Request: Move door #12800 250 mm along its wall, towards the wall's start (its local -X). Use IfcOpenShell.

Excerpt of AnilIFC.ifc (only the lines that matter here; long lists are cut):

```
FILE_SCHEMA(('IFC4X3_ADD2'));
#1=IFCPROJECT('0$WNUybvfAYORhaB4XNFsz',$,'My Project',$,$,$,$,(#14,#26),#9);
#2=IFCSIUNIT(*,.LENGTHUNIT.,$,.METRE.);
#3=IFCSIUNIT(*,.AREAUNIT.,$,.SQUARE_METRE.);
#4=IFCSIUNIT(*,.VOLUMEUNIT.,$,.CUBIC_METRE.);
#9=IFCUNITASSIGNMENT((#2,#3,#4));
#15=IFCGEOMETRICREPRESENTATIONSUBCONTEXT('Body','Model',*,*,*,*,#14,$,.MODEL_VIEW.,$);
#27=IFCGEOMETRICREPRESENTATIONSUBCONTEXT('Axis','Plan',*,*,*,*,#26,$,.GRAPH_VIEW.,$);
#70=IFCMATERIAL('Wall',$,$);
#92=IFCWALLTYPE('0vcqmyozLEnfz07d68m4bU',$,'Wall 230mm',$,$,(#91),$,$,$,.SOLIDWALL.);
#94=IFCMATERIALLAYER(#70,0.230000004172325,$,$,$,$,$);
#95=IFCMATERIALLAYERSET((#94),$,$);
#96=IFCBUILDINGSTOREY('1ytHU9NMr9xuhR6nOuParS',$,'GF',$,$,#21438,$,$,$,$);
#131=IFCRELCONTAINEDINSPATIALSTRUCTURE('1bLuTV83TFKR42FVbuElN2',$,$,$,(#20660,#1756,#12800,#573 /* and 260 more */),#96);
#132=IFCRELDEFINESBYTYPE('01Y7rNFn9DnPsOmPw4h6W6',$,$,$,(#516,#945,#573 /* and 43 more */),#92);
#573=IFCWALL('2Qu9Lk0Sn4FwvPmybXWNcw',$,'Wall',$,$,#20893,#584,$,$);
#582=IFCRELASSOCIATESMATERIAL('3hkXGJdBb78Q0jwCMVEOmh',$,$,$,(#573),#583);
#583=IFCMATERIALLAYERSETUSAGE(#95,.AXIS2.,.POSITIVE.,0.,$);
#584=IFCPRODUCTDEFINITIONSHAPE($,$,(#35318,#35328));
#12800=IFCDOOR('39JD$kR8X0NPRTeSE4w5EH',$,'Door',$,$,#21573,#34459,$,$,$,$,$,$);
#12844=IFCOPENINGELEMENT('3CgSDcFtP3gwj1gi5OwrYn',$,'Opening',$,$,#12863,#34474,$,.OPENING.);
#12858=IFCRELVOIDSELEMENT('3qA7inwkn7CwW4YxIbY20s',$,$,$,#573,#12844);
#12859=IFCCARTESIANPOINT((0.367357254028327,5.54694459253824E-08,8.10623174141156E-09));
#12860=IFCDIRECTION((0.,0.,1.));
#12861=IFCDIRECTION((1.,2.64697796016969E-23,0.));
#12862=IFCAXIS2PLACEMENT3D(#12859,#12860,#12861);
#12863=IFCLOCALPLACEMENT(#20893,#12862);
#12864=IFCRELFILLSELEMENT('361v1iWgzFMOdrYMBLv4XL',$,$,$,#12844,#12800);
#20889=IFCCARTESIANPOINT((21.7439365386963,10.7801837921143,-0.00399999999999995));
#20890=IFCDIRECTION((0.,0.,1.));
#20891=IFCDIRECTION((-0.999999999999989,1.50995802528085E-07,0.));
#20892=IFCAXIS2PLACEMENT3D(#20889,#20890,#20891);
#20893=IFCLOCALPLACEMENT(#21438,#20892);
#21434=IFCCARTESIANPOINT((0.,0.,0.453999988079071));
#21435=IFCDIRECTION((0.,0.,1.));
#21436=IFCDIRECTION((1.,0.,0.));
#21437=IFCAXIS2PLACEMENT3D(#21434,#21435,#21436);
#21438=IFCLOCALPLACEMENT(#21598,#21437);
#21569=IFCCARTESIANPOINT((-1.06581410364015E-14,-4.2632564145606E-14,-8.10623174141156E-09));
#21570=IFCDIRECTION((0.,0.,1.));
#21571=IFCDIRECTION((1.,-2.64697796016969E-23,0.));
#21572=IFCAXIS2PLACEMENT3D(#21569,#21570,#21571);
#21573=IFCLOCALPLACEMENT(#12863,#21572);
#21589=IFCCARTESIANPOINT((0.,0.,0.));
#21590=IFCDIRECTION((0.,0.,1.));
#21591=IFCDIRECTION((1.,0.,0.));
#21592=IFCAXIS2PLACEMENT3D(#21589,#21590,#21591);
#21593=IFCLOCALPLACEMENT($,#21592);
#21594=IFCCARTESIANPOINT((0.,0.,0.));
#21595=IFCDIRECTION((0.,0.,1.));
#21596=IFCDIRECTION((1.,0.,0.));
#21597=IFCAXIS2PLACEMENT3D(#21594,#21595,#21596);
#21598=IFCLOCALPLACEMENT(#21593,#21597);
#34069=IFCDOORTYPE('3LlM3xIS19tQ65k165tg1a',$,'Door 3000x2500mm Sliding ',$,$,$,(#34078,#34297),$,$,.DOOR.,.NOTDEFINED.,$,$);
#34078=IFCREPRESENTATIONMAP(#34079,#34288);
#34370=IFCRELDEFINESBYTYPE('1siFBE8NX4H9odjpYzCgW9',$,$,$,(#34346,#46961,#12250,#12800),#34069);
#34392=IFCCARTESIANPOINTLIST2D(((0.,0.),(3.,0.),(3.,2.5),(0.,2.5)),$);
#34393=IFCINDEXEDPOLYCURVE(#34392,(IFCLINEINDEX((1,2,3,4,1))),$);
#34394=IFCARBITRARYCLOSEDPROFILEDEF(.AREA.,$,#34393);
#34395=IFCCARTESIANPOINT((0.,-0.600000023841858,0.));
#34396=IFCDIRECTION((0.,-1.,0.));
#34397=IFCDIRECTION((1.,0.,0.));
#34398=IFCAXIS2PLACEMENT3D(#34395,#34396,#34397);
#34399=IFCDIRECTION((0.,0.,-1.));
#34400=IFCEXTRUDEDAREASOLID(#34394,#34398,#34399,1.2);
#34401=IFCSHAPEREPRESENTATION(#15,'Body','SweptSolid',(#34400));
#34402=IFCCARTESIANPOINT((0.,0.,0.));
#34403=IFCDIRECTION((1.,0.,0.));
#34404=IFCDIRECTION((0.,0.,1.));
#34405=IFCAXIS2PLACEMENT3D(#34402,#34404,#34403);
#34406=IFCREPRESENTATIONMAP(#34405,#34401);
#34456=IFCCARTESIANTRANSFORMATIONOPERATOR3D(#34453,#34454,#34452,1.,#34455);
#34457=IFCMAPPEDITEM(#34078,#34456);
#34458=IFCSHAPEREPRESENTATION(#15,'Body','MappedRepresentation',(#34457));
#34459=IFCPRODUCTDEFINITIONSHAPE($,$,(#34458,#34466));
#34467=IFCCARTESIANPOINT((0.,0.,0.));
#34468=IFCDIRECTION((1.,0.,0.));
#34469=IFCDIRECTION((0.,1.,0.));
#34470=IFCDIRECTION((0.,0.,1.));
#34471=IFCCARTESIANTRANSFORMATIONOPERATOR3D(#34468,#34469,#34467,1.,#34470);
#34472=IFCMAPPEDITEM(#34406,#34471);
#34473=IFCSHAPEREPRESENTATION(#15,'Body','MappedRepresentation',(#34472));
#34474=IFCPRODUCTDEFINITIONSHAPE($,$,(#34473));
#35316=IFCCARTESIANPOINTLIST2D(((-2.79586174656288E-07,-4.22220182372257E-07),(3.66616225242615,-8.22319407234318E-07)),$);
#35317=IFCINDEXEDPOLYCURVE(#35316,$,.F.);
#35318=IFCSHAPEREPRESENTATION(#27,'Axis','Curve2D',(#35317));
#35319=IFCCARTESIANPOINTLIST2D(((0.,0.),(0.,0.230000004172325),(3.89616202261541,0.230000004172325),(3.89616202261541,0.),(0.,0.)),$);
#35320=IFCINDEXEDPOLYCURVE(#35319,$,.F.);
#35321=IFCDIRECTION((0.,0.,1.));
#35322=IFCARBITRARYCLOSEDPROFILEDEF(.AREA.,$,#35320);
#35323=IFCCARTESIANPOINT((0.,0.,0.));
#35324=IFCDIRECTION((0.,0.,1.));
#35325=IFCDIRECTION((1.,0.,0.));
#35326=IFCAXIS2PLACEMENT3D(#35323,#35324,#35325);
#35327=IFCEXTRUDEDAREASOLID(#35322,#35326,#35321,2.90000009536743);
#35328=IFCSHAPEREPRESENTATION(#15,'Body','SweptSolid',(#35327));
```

```python
import ifcopenshell
import ifcopenshell.api.geometry
import ifcopenshell.util.placement
import ifcopenshell.util.unit

model = ifcopenshell.open("AnilIFC.ifc")
unit_scale = ifcopenshell.util.unit.calculate_unit_scale(model)

door = model.by_guid("39JD$kR8X0NPRTeSE4w5EH")
opening = door.FillsVoids[0].RelatingOpeningElement
wall = opening.VoidsElements[0].RelatingBuildingElement

wall_matrix = ifcopenshell.util.placement.get_local_placement(wall.ObjectPlacement)
shift = wall_matrix[:3, 0] * -0.25 / unit_scale
before = ifcopenshell.util.placement.get_local_placement(door.ObjectPlacement)[:3, 3].copy()

# The door is placed relative to its opening, so it follows when the opening moves.
matrix = ifcopenshell.util.placement.get_local_placement(opening.ObjectPlacement)
matrix[:3, 3] += shift
ifcopenshell.api.geometry.edit_object_placement(
    model, product=opening, matrix=matrix, is_si=False, should_transform_children=True
)

after = ifcopenshell.util.placement.get_local_placement(door.ObjectPlacement)[:3, 3]
print("door moved by", (after - before).round(3) + 0.0)

model.write("AnilIFC_v2.ifc")
```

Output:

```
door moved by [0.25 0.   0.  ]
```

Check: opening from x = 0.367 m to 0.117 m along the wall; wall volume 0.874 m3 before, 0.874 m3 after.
